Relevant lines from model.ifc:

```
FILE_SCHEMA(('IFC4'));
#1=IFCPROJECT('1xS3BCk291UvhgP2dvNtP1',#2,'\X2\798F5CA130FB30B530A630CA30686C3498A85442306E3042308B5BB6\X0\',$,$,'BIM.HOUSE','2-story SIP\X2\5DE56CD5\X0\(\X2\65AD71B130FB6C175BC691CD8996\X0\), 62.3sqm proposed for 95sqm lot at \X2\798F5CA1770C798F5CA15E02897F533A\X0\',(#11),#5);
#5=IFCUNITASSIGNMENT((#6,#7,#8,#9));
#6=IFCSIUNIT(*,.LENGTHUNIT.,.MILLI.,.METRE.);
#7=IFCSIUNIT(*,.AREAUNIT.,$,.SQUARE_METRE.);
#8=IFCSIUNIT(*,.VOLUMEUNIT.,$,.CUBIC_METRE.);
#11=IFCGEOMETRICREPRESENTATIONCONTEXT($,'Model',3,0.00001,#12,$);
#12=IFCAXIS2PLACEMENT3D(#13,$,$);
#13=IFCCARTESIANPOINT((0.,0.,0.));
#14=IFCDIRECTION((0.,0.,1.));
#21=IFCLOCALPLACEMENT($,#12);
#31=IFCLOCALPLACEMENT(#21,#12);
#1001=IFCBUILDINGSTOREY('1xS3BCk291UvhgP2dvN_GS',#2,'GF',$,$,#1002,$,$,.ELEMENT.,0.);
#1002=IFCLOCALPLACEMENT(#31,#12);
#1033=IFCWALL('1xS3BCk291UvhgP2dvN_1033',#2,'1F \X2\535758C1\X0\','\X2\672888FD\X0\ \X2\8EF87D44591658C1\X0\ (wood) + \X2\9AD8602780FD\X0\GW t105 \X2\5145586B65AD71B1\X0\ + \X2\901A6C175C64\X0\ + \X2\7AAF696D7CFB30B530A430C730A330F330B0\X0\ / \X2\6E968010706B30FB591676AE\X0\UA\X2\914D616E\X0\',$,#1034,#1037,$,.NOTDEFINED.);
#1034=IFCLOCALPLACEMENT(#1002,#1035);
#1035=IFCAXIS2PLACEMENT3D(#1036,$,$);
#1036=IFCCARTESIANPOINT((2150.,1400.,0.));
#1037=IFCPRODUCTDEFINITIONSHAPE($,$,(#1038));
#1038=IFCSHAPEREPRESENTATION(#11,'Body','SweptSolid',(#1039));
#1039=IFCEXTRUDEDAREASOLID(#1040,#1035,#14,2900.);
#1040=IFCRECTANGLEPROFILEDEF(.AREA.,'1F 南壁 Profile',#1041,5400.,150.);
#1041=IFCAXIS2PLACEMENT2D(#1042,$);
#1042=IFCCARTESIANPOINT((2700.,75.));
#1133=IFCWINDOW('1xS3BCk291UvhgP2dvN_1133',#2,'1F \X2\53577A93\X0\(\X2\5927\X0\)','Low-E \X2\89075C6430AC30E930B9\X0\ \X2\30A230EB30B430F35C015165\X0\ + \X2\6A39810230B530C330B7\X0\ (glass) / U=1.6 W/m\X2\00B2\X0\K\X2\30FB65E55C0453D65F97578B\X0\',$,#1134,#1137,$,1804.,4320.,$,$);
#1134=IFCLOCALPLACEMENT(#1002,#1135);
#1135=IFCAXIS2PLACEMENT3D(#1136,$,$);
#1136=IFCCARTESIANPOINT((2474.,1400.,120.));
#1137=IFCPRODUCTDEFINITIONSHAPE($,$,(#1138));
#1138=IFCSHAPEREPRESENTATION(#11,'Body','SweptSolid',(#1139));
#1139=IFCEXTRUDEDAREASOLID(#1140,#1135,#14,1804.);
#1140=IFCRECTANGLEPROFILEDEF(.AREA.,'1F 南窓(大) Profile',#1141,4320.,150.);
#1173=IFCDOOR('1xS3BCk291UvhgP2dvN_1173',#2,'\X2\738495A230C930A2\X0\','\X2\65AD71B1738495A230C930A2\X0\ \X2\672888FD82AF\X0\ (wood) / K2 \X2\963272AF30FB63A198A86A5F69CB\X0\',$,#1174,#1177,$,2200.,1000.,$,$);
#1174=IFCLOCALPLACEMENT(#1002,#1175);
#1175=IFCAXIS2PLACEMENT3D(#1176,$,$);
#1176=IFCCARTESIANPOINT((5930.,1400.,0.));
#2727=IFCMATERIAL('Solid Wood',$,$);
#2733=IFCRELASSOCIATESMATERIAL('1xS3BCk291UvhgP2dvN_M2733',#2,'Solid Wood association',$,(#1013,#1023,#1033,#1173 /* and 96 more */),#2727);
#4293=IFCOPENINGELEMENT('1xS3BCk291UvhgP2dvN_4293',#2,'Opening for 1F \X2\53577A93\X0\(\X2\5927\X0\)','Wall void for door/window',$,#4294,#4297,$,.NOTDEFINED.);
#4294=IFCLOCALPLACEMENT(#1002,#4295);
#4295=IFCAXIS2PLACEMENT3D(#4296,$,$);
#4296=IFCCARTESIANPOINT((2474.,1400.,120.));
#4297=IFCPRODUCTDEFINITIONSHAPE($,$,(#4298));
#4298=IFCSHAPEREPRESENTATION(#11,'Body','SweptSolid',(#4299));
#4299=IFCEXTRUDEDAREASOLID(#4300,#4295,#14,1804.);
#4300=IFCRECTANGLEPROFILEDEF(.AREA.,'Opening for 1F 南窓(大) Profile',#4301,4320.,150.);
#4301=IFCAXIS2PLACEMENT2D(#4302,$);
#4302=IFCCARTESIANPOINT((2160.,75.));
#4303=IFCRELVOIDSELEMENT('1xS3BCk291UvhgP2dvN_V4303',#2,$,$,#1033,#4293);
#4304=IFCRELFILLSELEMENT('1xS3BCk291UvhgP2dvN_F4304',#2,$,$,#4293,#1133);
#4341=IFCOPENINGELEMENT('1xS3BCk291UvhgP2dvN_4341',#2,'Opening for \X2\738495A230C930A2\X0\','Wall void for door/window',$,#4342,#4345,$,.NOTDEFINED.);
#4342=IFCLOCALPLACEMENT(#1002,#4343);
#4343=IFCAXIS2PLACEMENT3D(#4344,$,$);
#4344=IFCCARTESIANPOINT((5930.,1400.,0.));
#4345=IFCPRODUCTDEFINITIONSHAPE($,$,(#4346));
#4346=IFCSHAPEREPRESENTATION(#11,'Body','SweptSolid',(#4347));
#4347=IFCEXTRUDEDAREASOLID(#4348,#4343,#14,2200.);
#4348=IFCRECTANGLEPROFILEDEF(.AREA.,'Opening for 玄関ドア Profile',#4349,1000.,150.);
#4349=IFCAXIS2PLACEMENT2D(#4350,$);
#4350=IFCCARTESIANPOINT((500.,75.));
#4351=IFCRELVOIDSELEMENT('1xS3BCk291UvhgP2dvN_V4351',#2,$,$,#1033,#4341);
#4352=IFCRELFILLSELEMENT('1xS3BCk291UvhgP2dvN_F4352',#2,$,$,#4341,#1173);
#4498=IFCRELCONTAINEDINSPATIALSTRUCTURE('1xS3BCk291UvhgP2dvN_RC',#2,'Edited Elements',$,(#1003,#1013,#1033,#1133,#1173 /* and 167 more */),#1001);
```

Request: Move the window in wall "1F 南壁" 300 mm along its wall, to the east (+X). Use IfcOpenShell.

```python
import ifcopenshell
import ifcopenshell.api.geometry
import ifcopenshell.util.placement

model = ifcopenshell.open("model.ifc")

window = model.by_guid("1xS3BCk291UvhgP2dvN_1133")
opening = window.FillsVoids[0].RelatingOpeningElement
wall = opening.VoidsElements[0].RelatingBuildingElement

wall_matrix = ifcopenshell.util.placement.get_local_placement(wall.ObjectPlacement)
shift = wall_matrix[:3, 0] * 300.0
before = ifcopenshell.util.placement.get_local_placement(window.ObjectPlacement)[:3, 3].copy()

# The window is not placed relative to its opening, so move both.
for product in (opening, window):
    matrix = ifcopenshell.util.placement.get_local_placement(product.ObjectPlacement)
    matrix[:3, 3] += shift
    ifcopenshell.api.geometry.edit_object_placement(model, product=product, matrix=matrix, is_si=False)

after = ifcopenshell.util.placement.get_local_placement(window.ObjectPlacement)[:3, 3]
print("window moved by", (after - before).round(3) + 0.0)

model.write("model-out.ifc")
```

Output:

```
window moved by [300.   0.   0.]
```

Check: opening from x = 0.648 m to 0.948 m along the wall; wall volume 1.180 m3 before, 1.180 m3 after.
